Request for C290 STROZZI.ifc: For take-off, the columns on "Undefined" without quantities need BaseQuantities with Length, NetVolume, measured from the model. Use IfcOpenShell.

First a look at what the model holds.

```python
import ifcopenshell
import ifcopenshell.util.element
import ifcopenshell.util.unit

model = ifcopenshell.open("C290 STROZZI.ifc")
print(model.schema)
for unit_type in ("LENGTHUNIT", "AREAUNIT", "VOLUMEUNIT"):
    print(unit_type, ifcopenshell.util.unit.calculate_unit_scale(model, unit_type))
storey = next(s for s in model.by_type("IfcBuildingStorey") if s.Name == "Undefined")
columns = [e for e in ifcopenshell.util.element.get_decomposition(storey) if e.is_a("IfcColumn")]
for e in sorted(columns, key=lambda e: e.id()):
    print(e.id(), e.is_a(), e.Name, list(ifcopenshell.util.element.get_psets(e, qtos_only=True)), sep=" | ")
```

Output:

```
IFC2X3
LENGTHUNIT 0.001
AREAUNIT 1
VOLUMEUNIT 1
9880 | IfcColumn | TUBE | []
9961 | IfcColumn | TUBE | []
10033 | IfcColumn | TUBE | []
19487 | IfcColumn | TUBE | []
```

```python
import ifcopenshell
import ifcopenshell.api.pset
import ifcopenshell.geom
import ifcopenshell.util.element
import ifcopenshell.util.shape
import ifcopenshell.util.unit

model = ifcopenshell.open("C290 STROZZI.ifc")
unit_scale = ifcopenshell.util.unit.calculate_unit_scale(model)
volume_scale = ifcopenshell.util.unit.calculate_unit_scale(model, "VOLUMEUNIT")
settings = ifcopenshell.geom.settings()

storey = next(s for s in model.by_type("IfcBuildingStorey") if s.Name == "Undefined")
columns = [e for e in ifcopenshell.util.element.get_decomposition(storey) if e.is_a("IfcColumn")]

for e in sorted(columns, key=lambda e: e.id()):
    if ifcopenshell.util.element.get_psets(e, qtos_only=True, should_inherit=False):
        continue
    # Geometry comes back in metres, in the element's own axes.
    shape = ifcopenshell.geom.create_shape(settings, e)
    values = {
        "Length": ifcopenshell.util.shape.get_z(shape.geometry) / unit_scale,
        "NetVolume": ifcopenshell.util.shape.get_volume(shape.geometry) / volume_scale,
    }
    qto = ifcopenshell.api.pset.add_qto(model, product=e, name="BaseQuantities")
    ifcopenshell.api.pset.edit_qto(model, qto=qto, properties=values)
    print(e.id(), {k: round(v, 3) for k, v in values.items()})

model.write("C290 STROZZI-out.ifc")
```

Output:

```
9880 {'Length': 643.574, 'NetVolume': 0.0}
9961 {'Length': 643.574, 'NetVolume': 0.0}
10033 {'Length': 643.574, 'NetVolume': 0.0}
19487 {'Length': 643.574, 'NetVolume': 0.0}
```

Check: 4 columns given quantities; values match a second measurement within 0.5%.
